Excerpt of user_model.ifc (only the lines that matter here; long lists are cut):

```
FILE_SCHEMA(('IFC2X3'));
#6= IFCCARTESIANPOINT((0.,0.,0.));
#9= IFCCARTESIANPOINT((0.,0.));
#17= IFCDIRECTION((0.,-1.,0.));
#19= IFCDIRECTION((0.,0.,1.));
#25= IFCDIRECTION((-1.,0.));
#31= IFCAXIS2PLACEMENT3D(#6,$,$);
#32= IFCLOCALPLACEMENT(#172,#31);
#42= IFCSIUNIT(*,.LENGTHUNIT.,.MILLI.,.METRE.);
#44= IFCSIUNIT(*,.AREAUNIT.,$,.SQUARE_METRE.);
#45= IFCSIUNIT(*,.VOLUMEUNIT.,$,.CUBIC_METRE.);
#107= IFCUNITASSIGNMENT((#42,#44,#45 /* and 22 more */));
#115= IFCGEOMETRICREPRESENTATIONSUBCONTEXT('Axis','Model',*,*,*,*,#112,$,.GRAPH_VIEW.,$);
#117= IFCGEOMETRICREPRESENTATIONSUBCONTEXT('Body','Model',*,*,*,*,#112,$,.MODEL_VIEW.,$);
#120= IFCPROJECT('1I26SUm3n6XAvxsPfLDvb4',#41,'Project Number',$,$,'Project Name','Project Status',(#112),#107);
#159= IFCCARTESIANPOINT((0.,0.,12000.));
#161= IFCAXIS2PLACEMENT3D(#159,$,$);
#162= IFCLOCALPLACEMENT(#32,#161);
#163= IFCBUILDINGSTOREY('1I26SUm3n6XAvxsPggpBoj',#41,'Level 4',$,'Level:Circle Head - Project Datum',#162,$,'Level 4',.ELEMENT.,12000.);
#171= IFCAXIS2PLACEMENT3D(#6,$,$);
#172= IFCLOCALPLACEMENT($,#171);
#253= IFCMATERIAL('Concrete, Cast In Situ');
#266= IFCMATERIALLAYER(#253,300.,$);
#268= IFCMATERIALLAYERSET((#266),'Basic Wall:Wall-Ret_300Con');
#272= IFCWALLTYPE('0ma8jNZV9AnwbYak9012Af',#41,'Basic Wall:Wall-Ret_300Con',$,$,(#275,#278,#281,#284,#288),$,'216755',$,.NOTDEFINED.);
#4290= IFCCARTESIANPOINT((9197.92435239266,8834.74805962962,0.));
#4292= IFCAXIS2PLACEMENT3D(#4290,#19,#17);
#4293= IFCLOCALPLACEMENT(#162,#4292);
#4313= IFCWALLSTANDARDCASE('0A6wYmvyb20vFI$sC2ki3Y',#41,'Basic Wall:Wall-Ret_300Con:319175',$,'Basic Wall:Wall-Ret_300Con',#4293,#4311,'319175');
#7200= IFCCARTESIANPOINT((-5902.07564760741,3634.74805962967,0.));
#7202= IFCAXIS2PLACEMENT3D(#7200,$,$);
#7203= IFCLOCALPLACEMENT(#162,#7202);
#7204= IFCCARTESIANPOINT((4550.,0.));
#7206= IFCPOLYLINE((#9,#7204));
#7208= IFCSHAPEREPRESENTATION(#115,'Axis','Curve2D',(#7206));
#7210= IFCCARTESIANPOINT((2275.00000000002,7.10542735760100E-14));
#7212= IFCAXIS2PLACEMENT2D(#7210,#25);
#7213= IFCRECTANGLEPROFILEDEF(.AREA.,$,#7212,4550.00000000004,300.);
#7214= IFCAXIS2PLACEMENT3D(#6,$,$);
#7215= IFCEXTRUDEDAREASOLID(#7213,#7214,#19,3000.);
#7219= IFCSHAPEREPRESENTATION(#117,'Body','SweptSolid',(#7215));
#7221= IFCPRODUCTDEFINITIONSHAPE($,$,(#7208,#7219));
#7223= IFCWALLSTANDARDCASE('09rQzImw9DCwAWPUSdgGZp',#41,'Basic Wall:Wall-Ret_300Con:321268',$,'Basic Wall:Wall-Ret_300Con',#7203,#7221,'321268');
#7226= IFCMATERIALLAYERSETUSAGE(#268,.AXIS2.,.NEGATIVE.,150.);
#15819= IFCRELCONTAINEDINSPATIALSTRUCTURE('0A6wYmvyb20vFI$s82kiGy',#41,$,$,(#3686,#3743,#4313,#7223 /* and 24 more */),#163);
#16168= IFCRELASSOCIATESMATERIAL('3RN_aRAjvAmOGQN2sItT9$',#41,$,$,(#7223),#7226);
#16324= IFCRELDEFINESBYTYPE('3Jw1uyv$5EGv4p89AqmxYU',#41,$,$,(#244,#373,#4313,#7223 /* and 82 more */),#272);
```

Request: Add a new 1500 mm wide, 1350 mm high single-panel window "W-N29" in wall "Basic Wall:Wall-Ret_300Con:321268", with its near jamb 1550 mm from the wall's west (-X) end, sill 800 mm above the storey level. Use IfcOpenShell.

```python
import numpy as np
import ifcopenshell
import ifcopenshell.api.feature
import ifcopenshell.api.geometry
import ifcopenshell.api.root
import ifcopenshell.api.spatial
import ifcopenshell.api.type
import ifcopenshell.geom
import ifcopenshell.util.element
import ifcopenshell.util.placement
import ifcopenshell.util.representation
import ifcopenshell.util.shape
import ifcopenshell.util.unit

model = ifcopenshell.open("user_model.ifc")
unit_scale = ifcopenshell.util.unit.calculate_unit_scale(model)
settings = ifcopenshell.geom.settings()


def volume(element):
    """Net volume in cubic metres, openings subtracted."""
    shape = ifcopenshell.geom.create_shape(settings, element)
    return ifcopenshell.util.shape.get_volume(shape.geometry)


wall = model.by_id(7223)
storey = ifcopenshell.util.element.get_container(wall, ifc_class="IfcBuildingStorey")
context = ifcopenshell.util.representation.get_context(model, "Model", "Body", "MODEL_VIEW")
before = volume(wall)

width, height, from_end, sill = 1.5, 1.35, 1.55, 0.8  # metres

# The wall runs along its own X axis, and the end named is its -X end.
wall_shape = ifcopenshell.geom.create_shape(settings, wall)
x, y, z = ifcopenshell.util.shape.get_vertices(wall_shape.geometry).T
start = x.min() + from_end
face, thickness = float(y.min()), float(y.max() - y.min())
wall_matrix = ifcopenshell.util.placement.get_local_placement(wall.ObjectPlacement)
level = ifcopenshell.util.placement.get_local_placement(storey.ObjectPlacement)[2, 3]


def in_wall(x, y):
    """Placement at x, y metres in the wall's axes, at sill height."""
    matrix = wall_matrix.copy()
    matrix[:, 3] = wall_matrix @ np.array([x / unit_scale, y / unit_scale, 0.0, 1.0])
    matrix[2, 3] = level + sill / unit_scale
    return matrix


# Opening: a box that overshoots both wall faces by 50 mm.
opening = ifcopenshell.api.root.create_entity(model, ifc_class="IfcOpeningElement")
box = ifcopenshell.api.geometry.add_wall_representation(
    model, context=context, length=width, height=height, thickness=thickness + 0.1
)
ifcopenshell.api.geometry.assign_representation(model, product=opening, representation=box)
ifcopenshell.api.geometry.edit_object_placement(model, product=opening, matrix=in_wall(start, face - 0.05), is_si=False)
ifcopenshell.api.feature.add_feature(model, feature=opening, element=wall)

window = ifcopenshell.api.root.create_entity(model, ifc_class="IfcWindow", name="W-N29")
window.OverallWidth, window.OverallHeight = width / unit_scale, height / unit_scale
body = ifcopenshell.api.geometry.add_window_representation(
    model,
    context=context,
    overall_width=window.OverallWidth,
    overall_height=window.OverallHeight,
    partition_type="SINGLE_PANEL",
)
ifcopenshell.api.geometry.assign_representation(model, product=window, representation=body)
ifcopenshell.api.spatial.assign_container(model, products=[window], relating_structure=storey)
fills = ifcopenshell.api.feature.add_filling(model, opening=opening, element=window)
fills.OwnerHistory = window.OwnerHistory  # required in IFC2X3

# IFC2X3 keeps the operation on the window style.
style = ifcopenshell.api.root.create_entity(model, ifc_class="IfcWindowStyle", name="W-N29")
style.OperationType, style.ConstructionType = "SINGLE_PANEL", "NOTDEFINED"
style.ParameterTakesPrecedence = style.Sizeable = False
ifcopenshell.api.type.assign_type(model, related_objects=[window], relating_type=style)

# Centre the window in the wall's thickness.
ifcopenshell.api.geometry.edit_object_placement(model, product=window, matrix=in_wall(start, face), is_si=False)
window_shape = ifcopenshell.geom.create_shape(settings, window)
depth = ifcopenshell.util.shape.get_vertices(window_shape.geometry)[:, 1]
offset = face + thickness / 2 - (depth.min() + depth.max()) / 2
ifcopenshell.api.geometry.edit_object_placement(model, product=window, matrix=in_wall(start, offset), is_si=False)

after = volume(wall)

print(f"wall volume {before:.3f} -> {after:.3f} m3")

model.write("user_model_updated.ifc")
```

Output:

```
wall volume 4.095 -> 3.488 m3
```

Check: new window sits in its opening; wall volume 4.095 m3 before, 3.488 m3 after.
